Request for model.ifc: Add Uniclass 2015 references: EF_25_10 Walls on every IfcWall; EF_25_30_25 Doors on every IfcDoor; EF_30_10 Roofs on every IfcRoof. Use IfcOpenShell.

First a look at what the model holds.

```python
import ifcopenshell

model = ifcopenshell.open("model.ifc")
print(model.schema)
print("classifications:", [c.Name for c in model.by_type("IfcClassification")])
for ifc_class in ("IfcDoor", "IfcRoof", "IfcStair", "IfcWall", "IfcWindow"):
    print(ifc_class, len(model.by_type(ifc_class)))
```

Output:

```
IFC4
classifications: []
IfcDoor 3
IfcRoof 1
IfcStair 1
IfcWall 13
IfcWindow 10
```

```python
import ifcopenshell
import ifcopenshell.api.classification

model = ifcopenshell.open("model.ifc")

system = ifcopenshell.api.classification.add_classification(model, classification="Uniclass 2015")

codes = {
    "IfcWall": ("EF_25_10", "Walls"),
    "IfcDoor": ("EF_25_30_25", "Doors"),
    "IfcRoof": ("EF_30_10", "Roofs"),
}
for ifc_class, (code, name) in codes.items():
    products = model.by_type(ifc_class)
    ifcopenshell.api.classification.add_reference(
        model, products=products, classification=system, identification=code, name=name
    )
    print(code, len(products))

model.write("model_edited.ifc")
```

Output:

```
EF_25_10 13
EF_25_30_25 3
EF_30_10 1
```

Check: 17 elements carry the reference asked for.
